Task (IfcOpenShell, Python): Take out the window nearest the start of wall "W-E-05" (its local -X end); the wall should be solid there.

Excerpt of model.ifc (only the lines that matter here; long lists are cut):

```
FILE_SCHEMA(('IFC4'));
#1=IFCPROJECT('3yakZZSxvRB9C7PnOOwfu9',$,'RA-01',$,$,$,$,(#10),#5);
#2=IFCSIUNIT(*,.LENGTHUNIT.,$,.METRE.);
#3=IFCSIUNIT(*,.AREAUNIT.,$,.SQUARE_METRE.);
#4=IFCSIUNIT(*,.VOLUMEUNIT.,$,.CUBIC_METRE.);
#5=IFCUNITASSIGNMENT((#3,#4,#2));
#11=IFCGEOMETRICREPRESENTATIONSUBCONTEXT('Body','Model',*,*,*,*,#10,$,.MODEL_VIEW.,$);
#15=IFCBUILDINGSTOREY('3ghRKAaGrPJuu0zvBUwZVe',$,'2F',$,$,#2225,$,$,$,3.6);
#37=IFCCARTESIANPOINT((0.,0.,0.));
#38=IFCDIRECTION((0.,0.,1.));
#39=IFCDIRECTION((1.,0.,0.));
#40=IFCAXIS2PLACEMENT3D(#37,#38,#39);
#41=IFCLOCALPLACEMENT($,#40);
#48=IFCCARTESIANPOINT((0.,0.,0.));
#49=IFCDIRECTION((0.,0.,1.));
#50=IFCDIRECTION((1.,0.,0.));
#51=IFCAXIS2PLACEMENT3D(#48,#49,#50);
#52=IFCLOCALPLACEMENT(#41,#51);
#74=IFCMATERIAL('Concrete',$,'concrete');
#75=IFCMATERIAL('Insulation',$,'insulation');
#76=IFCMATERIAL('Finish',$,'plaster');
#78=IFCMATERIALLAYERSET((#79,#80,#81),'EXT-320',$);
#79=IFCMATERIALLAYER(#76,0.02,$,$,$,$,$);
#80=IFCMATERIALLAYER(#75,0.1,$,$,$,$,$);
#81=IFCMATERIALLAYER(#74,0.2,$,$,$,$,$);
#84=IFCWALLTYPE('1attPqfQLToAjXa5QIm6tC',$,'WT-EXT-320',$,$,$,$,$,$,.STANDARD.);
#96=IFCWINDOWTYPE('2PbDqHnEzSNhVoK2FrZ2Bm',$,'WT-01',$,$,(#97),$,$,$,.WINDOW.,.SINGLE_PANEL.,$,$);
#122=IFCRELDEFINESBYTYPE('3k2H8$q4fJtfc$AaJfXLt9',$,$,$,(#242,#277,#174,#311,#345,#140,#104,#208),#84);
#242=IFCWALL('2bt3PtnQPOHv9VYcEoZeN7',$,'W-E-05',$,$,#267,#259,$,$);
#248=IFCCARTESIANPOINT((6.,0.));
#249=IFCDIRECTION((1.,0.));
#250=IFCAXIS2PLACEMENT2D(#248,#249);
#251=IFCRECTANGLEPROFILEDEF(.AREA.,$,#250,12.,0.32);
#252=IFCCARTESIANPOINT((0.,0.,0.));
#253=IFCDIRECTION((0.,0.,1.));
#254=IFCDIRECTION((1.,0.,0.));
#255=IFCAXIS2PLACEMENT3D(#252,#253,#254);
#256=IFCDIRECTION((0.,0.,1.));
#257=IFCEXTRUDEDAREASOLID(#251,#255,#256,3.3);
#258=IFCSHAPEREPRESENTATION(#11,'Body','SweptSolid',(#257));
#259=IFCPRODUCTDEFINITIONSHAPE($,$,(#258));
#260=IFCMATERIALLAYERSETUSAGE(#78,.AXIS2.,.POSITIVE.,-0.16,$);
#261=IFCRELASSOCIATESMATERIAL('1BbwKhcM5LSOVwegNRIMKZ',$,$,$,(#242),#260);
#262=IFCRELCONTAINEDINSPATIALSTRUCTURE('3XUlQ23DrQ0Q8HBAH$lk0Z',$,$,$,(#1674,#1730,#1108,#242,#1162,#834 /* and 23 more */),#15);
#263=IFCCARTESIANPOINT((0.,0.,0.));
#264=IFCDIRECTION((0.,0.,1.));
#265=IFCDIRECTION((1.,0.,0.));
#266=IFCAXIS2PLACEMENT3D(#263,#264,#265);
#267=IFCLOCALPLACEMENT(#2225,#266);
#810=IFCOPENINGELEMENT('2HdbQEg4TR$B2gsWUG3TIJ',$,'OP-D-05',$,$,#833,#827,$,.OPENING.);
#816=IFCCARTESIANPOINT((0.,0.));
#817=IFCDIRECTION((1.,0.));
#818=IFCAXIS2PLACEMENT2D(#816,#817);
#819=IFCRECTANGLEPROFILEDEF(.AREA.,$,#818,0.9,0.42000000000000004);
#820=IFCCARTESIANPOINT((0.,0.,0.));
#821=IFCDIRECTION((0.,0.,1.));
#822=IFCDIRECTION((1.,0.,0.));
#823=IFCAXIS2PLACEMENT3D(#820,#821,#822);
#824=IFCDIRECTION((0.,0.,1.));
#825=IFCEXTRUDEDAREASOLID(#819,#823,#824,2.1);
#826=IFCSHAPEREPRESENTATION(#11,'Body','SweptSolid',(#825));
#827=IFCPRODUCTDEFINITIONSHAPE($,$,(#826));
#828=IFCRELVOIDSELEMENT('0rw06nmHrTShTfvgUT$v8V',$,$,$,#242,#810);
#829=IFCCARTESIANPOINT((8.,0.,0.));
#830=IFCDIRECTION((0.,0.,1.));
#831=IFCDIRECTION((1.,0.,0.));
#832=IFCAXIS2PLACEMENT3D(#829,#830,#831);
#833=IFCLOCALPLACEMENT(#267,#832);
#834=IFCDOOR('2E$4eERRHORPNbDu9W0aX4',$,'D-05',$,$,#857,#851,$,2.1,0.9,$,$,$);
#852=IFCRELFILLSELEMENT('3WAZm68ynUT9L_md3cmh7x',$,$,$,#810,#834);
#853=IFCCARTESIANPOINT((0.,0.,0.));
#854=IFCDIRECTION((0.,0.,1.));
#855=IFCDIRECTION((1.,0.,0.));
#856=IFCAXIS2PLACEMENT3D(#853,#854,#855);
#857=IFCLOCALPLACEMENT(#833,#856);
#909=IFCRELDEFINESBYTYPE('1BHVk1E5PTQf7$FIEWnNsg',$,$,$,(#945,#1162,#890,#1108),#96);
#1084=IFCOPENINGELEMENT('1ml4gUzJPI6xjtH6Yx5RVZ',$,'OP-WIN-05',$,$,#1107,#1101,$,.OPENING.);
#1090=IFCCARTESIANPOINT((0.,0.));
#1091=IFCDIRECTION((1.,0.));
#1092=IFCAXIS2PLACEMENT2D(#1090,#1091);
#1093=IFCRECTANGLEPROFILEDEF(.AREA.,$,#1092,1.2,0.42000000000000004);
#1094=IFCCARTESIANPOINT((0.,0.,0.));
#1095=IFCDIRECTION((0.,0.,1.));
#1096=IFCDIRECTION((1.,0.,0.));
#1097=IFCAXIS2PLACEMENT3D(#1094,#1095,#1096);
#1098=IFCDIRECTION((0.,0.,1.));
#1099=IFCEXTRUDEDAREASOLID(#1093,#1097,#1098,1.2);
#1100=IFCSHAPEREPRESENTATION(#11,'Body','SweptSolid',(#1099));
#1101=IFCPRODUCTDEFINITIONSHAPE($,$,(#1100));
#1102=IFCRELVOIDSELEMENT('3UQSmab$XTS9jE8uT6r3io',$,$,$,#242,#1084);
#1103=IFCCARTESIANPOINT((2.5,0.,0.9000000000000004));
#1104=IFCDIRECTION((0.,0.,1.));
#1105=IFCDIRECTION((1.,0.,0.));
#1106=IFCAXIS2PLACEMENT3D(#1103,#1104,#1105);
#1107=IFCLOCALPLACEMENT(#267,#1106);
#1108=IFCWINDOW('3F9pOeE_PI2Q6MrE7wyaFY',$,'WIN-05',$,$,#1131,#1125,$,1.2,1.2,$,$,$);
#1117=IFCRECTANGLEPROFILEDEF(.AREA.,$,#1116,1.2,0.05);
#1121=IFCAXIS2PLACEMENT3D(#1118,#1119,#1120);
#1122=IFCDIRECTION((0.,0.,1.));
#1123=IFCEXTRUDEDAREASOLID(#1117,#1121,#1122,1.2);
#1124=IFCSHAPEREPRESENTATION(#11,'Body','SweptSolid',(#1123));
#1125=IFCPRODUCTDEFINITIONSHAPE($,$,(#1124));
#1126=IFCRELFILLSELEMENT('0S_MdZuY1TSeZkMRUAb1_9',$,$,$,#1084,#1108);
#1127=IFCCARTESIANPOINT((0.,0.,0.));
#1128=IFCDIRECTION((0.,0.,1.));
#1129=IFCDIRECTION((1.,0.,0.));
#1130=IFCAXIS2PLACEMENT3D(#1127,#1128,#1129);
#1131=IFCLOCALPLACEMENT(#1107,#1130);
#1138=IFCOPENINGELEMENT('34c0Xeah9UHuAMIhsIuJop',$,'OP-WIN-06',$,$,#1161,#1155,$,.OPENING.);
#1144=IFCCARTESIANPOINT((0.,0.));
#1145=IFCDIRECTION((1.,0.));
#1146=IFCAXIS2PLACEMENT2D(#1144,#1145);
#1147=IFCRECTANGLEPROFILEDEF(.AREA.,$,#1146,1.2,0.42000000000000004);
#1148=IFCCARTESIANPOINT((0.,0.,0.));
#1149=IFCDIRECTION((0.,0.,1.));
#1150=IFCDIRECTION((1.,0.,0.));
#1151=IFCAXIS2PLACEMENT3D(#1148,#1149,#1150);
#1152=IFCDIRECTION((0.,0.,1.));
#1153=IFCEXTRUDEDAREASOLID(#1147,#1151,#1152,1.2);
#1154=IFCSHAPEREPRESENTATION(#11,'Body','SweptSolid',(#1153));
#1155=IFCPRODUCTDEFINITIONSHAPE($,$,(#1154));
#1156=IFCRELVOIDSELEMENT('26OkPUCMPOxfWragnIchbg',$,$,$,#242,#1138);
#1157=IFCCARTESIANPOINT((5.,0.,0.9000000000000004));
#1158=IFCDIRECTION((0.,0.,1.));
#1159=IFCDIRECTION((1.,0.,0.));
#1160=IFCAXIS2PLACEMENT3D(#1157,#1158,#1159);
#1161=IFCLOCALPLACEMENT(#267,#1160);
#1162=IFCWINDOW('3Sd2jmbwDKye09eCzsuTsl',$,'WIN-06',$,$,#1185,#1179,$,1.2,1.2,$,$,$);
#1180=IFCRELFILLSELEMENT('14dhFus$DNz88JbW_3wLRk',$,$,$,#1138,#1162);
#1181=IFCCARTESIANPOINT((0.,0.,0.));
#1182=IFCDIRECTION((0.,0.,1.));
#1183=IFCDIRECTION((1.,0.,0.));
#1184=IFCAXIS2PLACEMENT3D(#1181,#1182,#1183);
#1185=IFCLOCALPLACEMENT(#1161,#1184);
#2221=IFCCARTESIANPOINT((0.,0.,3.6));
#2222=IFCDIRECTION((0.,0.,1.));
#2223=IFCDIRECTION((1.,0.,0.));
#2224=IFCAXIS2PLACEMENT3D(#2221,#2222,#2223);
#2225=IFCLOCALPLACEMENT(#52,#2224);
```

```python
import ifcopenshell
import ifcopenshell.api.feature
import ifcopenshell.api.root
import ifcopenshell.geom
import ifcopenshell.util.shape

model = ifcopenshell.open("model.ifc")
settings = ifcopenshell.geom.settings()


def volume(element):
    """Net volume in cubic metres, openings subtracted."""
    shape = ifcopenshell.geom.create_shape(settings, element)
    return ifcopenshell.util.shape.get_volume(shape.geometry)


window = model.by_guid("3F9pOeE_PI2Q6MrE7wyaFY")
opening = window.FillsVoids[0].RelatingOpeningElement
wall = opening.VoidsElements[0].RelatingBuildingElement
before = volume(wall)

ifcopenshell.api.root.remove_product(model, product=window)
ifcopenshell.api.feature.remove_feature(model, feature=opening)

after = volume(wall)

print(f"wall volume {before:.3f} -> {after:.3f} m3")

model.write("model-out.ifc")
```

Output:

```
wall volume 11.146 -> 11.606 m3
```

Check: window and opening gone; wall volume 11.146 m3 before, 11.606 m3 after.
